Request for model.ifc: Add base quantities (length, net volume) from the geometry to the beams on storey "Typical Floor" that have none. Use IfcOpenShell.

First a look at what the model holds.

```python
import ifcopenshell
import ifcopenshell.util.element
import ifcopenshell.util.unit

model = ifcopenshell.open("model.ifc")
print(model.schema)
for unit_type in ("LENGTHUNIT", "AREAUNIT", "VOLUMEUNIT"):
    print(unit_type, ifcopenshell.util.unit.calculate_unit_scale(model, unit_type))
storey = next(s for s in model.by_type("IfcBuildingStorey") if s.Name == "Typical Floor")
beams = [e for e in ifcopenshell.util.element.get_decomposition(storey) if e.is_a("IfcBeam")]
for e in sorted(beams, key=lambda e: e.id()):
    print(e.id(), e.is_a(), e.Name, list(ifcopenshell.util.element.get_psets(e, qtos_only=True)), sep=" | ")
```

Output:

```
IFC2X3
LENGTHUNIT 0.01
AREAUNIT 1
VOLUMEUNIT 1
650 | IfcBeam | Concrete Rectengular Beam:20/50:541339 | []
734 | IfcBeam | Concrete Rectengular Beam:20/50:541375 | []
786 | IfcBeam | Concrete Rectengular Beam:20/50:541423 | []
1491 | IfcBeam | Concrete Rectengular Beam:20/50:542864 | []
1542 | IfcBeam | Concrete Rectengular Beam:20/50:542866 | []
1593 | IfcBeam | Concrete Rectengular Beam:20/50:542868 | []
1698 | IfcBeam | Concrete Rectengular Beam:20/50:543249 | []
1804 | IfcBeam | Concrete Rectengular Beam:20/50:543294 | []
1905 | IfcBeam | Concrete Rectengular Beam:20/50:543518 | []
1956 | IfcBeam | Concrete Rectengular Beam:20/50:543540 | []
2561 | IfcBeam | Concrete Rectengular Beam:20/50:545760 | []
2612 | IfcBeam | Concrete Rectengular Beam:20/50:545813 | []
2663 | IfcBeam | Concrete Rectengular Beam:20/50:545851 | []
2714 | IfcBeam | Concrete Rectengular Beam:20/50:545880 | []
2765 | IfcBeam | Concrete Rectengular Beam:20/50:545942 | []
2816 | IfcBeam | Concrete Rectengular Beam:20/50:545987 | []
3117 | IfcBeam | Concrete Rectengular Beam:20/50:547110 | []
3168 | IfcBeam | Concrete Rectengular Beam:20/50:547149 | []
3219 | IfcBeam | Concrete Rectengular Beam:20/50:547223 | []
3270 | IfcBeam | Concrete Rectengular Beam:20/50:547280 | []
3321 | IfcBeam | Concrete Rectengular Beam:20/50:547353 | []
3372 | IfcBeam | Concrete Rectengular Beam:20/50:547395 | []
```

```python
import ifcopenshell
import ifcopenshell.api.pset
import ifcopenshell.geom
import ifcopenshell.util.element
import ifcopenshell.util.shape
import ifcopenshell.util.unit

model = ifcopenshell.open("model.ifc")
unit_scale = ifcopenshell.util.unit.calculate_unit_scale(model)
volume_scale = ifcopenshell.util.unit.calculate_unit_scale(model, "VOLUMEUNIT")
settings = ifcopenshell.geom.settings()

storey = next(s for s in model.by_type("IfcBuildingStorey") if s.Name == "Typical Floor")
beams = [e for e in ifcopenshell.util.element.get_decomposition(storey) if e.is_a("IfcBeam")]

for e in sorted(beams, key=lambda e: e.id()):
    if ifcopenshell.util.element.get_psets(e, qtos_only=True, should_inherit=False):
        continue
    # Geometry comes back in metres, in the element's own axes.
    shape = ifcopenshell.geom.create_shape(settings, e)
    values = {
        "Length": ifcopenshell.util.shape.get_max_xyz(shape.geometry) / unit_scale,
        "NetVolume": ifcopenshell.util.shape.get_volume(shape.geometry) / volume_scale,
    }
    qto = ifcopenshell.api.pset.add_qto(model, product=e, name="BaseQuantities")
    ifcopenshell.api.pset.edit_qto(model, qto=qto, properties=values)
    print(e.id(), {k: round(v, 3) for k, v in values.items()})

model.write("model-out.ifc")
```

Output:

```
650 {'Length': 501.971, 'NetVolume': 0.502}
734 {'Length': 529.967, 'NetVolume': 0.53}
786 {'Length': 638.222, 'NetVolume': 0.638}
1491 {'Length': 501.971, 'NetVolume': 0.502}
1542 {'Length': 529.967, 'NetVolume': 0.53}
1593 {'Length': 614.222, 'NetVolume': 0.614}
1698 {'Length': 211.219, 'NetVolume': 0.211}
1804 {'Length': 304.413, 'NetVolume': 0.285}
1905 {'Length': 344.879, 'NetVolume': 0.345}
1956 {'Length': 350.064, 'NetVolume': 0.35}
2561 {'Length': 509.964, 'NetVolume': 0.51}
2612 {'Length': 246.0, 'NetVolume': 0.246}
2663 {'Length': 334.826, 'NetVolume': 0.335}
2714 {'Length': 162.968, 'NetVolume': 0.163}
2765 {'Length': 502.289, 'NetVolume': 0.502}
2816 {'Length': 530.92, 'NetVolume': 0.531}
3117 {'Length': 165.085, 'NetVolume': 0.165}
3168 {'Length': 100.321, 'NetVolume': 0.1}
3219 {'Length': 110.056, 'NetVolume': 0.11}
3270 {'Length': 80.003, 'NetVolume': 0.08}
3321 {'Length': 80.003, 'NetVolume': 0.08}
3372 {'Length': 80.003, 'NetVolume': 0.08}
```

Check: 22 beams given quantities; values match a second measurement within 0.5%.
